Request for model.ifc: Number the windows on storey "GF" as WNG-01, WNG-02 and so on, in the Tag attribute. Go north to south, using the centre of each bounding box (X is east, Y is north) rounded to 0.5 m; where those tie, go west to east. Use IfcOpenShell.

First a look at what the model holds.

```python
import ifcopenshell
import ifcopenshell.util.element
import ifcopenshell.util.placement

model = ifcopenshell.open("model.ifc")
print(model.schema)
storey = next(s for s in model.by_type("IfcBuildingStorey") if s.Name == "GF")
windows = [e for e in ifcopenshell.util.element.get_decomposition(storey) if e.is_a("IfcWindow")]
for e in sorted(windows, key=lambda e: e.id()):
    origin = ifcopenshell.util.placement.get_local_placement(e.ObjectPlacement)[:3, 3]
    print(e.id(), e.Tag, e.Name, origin.round(2) + 0.0, sep=" | ")
```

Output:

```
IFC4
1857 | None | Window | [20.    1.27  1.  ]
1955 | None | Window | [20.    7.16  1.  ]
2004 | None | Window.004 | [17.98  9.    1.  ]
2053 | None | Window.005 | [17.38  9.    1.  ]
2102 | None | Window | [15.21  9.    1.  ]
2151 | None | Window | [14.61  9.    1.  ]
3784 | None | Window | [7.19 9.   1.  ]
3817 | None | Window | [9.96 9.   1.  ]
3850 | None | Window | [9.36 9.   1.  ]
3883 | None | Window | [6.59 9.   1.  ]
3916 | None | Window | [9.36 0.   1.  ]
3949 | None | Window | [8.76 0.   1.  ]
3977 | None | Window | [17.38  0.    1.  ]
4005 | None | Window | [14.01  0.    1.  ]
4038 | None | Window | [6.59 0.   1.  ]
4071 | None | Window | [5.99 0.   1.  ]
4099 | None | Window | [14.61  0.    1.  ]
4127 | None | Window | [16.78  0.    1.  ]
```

```python
import ifcopenshell
import ifcopenshell.geom
import ifcopenshell.util.element
import ifcopenshell.util.shape

model = ifcopenshell.open("model.ifc")
settings = ifcopenshell.geom.settings()
settings.set("use-world-coords", True)


def centre(element):
    shape = ifcopenshell.geom.create_shape(settings, element)
    return ifcopenshell.util.shape.get_bbox_centroid(shape.geometry)


storey = next(s for s in model.by_type("IfcBuildingStorey") if s.Name == "GF")
windows = [e for e in ifcopenshell.util.element.get_decomposition(storey) if e.is_a("IfcWindow")]

# Insertion points can sit at a corner or the storey origin, so sort by the geometry (in metres).
centres = {e: centre(e) for e in windows}
windows.sort(key=lambda e: (-round(centres[e][1] / 0.5), centres[e][0]))

for i, e in enumerate(windows, start=1):
    number = f"WNG-{i:02d}"
    e.Tag = number
    print(e.id(), number)

model.write("model-out.ifc")
```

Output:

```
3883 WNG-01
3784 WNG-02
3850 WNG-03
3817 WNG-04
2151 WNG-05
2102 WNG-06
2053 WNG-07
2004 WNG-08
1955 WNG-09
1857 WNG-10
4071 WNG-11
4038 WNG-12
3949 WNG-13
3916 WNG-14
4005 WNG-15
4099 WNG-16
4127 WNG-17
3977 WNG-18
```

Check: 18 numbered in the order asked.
